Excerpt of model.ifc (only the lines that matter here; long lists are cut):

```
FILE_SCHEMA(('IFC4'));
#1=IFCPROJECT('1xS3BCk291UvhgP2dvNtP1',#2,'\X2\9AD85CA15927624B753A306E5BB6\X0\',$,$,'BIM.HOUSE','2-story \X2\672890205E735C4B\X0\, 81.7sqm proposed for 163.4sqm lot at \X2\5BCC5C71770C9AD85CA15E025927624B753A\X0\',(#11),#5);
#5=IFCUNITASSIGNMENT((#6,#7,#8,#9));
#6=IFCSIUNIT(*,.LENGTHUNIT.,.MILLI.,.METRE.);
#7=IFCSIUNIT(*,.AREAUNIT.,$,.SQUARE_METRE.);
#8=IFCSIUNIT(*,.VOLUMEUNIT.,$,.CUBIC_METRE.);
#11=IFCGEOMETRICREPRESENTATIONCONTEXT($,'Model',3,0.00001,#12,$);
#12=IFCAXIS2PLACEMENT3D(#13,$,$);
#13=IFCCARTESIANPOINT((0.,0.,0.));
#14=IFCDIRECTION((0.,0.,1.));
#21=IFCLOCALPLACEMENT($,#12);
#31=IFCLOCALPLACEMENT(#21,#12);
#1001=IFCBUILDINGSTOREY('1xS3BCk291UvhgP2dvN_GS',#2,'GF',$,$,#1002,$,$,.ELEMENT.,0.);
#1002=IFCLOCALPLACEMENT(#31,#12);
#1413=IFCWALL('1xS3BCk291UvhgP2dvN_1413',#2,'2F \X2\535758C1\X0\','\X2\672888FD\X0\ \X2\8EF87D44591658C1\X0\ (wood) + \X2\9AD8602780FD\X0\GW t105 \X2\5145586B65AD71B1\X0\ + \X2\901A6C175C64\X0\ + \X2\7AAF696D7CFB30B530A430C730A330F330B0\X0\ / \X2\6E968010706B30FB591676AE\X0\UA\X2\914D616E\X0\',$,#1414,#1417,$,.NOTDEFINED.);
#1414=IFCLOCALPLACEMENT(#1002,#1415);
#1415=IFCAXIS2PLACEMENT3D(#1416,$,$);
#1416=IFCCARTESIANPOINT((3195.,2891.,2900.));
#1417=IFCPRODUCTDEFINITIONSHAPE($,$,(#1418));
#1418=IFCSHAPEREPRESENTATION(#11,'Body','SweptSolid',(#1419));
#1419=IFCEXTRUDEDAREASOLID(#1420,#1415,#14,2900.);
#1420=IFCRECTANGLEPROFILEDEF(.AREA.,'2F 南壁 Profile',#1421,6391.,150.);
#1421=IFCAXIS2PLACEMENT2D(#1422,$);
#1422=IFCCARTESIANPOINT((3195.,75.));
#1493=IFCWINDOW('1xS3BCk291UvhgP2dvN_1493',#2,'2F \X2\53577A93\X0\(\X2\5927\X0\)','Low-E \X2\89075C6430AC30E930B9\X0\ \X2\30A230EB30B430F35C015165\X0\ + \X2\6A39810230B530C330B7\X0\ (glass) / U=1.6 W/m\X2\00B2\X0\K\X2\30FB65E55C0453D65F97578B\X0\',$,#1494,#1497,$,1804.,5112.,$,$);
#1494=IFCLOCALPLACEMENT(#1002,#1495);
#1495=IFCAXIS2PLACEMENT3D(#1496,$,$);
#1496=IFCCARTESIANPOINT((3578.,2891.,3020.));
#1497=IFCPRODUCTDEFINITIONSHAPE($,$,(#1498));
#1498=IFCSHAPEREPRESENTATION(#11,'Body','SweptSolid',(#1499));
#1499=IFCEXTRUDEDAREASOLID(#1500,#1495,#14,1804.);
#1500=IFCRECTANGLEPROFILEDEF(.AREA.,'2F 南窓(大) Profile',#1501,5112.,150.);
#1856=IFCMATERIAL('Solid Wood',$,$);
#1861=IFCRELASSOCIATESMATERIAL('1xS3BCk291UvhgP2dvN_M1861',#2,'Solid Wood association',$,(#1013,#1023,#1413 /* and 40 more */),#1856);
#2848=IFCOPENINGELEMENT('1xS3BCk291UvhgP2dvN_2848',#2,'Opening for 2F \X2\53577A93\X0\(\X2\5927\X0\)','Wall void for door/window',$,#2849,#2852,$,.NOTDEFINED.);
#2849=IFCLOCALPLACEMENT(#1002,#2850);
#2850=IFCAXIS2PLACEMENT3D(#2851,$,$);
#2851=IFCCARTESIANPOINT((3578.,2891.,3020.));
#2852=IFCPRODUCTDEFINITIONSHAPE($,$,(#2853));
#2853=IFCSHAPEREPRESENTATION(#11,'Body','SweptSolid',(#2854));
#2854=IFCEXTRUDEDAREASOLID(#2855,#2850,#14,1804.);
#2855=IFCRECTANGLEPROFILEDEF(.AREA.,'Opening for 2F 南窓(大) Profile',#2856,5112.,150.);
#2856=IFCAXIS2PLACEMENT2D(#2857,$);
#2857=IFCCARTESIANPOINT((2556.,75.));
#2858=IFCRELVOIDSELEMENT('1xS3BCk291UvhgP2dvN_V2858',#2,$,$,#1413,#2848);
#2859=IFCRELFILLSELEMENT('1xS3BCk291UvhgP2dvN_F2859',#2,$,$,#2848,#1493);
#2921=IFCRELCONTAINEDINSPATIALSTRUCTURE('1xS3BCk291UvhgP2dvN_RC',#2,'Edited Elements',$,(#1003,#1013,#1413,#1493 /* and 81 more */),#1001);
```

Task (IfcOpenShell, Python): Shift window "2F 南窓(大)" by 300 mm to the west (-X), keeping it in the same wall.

```python
import ifcopenshell
import ifcopenshell.api.geometry
import ifcopenshell.util.placement
import ifcopenshell.util.unit

model = ifcopenshell.open("model.ifc")
unit_scale = ifcopenshell.util.unit.calculate_unit_scale(model)

window = model.by_guid("1xS3BCk291UvhgP2dvN_1493")
opening = window.FillsVoids[0].RelatingOpeningElement
wall = opening.VoidsElements[0].RelatingBuildingElement

wall_matrix = ifcopenshell.util.placement.get_local_placement(wall.ObjectPlacement)
shift = wall_matrix[:3, 0] * -0.3 / unit_scale
before = ifcopenshell.util.placement.get_local_placement(window.ObjectPlacement)[:3, 3].copy()

# The window is not placed relative to its opening, so move both.
for product in (opening, window):
    matrix = ifcopenshell.util.placement.get_local_placement(product.ObjectPlacement)
    matrix[:3, 3] += shift
    ifcopenshell.api.geometry.edit_object_placement(model, product=product, matrix=matrix, is_si=False)

after = ifcopenshell.util.placement.get_local_placement(window.ObjectPlacement)[:3, 3]
print("window moved by", (after - before).round(3) + 0.0)

model.write("model_updated.ifc")
```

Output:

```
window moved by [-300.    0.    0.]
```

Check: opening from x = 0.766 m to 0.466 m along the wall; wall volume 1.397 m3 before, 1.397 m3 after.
